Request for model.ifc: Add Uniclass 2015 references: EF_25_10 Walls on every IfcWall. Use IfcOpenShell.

First a look at what the model holds.

```python
import ifcopenshell

model = ifcopenshell.open("model.ifc")
print(model.schema)
print("classifications:", [c.Name for c in model.by_type("IfcClassification")])
for ifc_class in ("IfcDoor", "IfcRoof", "IfcStair", "IfcWall", "IfcWindow"):
    print(ifc_class, len(model.by_type(ifc_class)))
```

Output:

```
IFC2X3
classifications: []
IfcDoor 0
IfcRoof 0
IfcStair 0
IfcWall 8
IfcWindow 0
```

```python
import ifcopenshell
import ifcopenshell.api.classification

model = ifcopenshell.open("model.ifc")

# IFC2X3 requires Source and Edition and has no link from the project to the system.
system = model.create_entity("IfcClassification", Source="NBS", Edition="2015", Name="Uniclass 2015")

codes = {
    "IfcWall": ("EF_25_10", "Walls"),
}
for ifc_class, (code, name) in codes.items():
    products = model.by_type(ifc_class)
    ifcopenshell.api.classification.add_reference(
        model, products=products, classification=system, identification=code, name=name
    )
    print(code, len(products))

model.write("model-out.ifc")
```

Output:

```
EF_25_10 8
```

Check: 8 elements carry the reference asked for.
